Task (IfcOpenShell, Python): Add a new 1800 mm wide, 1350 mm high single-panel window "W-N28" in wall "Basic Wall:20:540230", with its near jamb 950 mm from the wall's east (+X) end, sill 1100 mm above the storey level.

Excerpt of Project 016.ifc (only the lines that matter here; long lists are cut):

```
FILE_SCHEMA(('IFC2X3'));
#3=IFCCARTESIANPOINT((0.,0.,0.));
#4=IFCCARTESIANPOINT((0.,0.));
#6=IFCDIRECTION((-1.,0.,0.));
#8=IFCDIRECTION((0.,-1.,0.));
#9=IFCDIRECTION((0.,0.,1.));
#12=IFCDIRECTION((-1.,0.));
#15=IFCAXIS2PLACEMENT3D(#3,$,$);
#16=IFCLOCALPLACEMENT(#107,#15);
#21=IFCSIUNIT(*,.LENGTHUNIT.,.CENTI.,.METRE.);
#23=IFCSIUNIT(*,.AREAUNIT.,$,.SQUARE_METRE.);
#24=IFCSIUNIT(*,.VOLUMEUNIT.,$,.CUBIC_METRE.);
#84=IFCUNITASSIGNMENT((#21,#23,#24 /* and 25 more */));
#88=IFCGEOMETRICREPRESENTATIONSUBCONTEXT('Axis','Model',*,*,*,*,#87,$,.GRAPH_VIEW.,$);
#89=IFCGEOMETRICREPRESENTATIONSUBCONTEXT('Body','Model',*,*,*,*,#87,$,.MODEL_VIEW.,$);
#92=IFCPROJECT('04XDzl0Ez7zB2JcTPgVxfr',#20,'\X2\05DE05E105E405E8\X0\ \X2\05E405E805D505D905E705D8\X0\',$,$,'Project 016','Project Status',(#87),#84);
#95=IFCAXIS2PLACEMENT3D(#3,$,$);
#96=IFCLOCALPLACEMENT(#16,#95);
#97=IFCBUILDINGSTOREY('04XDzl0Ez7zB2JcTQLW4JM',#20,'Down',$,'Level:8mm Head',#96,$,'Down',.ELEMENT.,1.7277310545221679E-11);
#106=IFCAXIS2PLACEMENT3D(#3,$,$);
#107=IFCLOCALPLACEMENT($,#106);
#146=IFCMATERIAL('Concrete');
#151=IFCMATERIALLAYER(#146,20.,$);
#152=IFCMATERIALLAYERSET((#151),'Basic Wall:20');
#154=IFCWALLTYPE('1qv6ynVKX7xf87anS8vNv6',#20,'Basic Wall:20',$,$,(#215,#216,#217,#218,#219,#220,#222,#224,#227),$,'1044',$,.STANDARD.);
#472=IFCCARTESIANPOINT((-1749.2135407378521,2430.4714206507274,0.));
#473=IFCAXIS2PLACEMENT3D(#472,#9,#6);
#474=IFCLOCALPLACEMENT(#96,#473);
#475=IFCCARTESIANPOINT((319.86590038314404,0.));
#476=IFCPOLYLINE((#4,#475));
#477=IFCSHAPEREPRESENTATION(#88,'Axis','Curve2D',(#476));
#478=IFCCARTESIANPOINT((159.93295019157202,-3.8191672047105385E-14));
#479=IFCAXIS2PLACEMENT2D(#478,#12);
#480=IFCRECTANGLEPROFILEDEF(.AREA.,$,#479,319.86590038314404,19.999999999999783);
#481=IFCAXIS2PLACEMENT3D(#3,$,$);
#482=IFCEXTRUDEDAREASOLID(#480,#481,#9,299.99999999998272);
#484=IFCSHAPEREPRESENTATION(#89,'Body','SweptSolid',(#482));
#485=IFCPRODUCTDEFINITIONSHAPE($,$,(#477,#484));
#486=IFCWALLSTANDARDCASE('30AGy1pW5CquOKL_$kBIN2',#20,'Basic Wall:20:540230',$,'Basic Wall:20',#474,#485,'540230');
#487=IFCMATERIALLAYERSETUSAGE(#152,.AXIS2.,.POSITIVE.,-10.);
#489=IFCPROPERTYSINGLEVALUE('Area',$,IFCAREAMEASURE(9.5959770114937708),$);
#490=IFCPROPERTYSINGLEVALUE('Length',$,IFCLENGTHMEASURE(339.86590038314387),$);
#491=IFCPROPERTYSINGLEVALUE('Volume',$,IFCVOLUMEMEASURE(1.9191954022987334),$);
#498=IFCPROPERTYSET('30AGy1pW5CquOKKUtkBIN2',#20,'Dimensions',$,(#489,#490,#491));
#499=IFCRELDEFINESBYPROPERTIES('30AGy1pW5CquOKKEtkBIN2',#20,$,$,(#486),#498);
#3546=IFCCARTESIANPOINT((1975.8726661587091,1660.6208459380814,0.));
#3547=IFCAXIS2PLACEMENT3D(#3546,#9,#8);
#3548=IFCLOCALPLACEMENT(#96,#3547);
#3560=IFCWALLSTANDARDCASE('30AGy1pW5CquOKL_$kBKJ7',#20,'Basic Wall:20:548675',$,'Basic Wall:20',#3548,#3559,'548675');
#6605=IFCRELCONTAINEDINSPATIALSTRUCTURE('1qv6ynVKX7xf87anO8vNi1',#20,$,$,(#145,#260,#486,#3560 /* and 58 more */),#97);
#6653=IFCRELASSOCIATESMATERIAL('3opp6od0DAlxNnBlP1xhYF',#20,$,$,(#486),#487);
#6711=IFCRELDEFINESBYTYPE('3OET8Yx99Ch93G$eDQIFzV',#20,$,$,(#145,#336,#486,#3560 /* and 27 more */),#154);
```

```python
import numpy as np
import ifcopenshell
import ifcopenshell.api.feature
import ifcopenshell.api.geometry
import ifcopenshell.api.pset
import ifcopenshell.api.root
import ifcopenshell.api.spatial
import ifcopenshell.api.type
import ifcopenshell.geom
import ifcopenshell.util.element
import ifcopenshell.util.placement
import ifcopenshell.util.representation
import ifcopenshell.util.shape
import ifcopenshell.util.unit

model = ifcopenshell.open("Project 016.ifc")
unit_scale = ifcopenshell.util.unit.calculate_unit_scale(model)
area_scale = ifcopenshell.util.unit.calculate_unit_scale(model, "AREAUNIT")
volume_scale = ifcopenshell.util.unit.calculate_unit_scale(model, "VOLUMEUNIT")
settings = ifcopenshell.geom.settings()


def volume(element):
    """Net volume in cubic metres, openings subtracted."""
    shape = ifcopenshell.geom.create_shape(settings, element)
    return ifcopenshell.util.shape.get_volume(shape.geometry)


wall = model.by_id(486)
storey = ifcopenshell.util.element.get_container(wall, ifc_class="IfcBuildingStorey")
context = ifcopenshell.util.representation.get_context(model, "Model", "Body", "MODEL_VIEW")
before = volume(wall)

width, height, from_end, sill = 1.8, 1.35, 0.95, 1.1  # metres

# The wall runs along its own X axis, and the end named is its -X end.
wall_shape = ifcopenshell.geom.create_shape(settings, wall)
x, y, z = ifcopenshell.util.shape.get_vertices(wall_shape.geometry).T
start = x.min() + from_end
face, thickness = float(y.min()), float(y.max() - y.min())
wall_matrix = ifcopenshell.util.placement.get_local_placement(wall.ObjectPlacement)
level = ifcopenshell.util.placement.get_local_placement(storey.ObjectPlacement)[2, 3]


def in_wall(x, y):
    """Placement at x, y metres in the wall's axes, at sill height."""
    matrix = wall_matrix.copy()
    matrix[:, 3] = wall_matrix @ np.array([x / unit_scale, y / unit_scale, 0.0, 1.0])
    matrix[2, 3] = level + sill / unit_scale
    return matrix


# Opening: a box that overshoots both wall faces by 50 mm.
opening = ifcopenshell.api.root.create_entity(model, ifc_class="IfcOpeningElement")
box = ifcopenshell.api.geometry.add_wall_representation(
    model, context=context, length=width, height=height, thickness=thickness + 0.1
)
ifcopenshell.api.geometry.assign_representation(model, product=opening, representation=box)
ifcopenshell.api.geometry.edit_object_placement(model, product=opening, matrix=in_wall(start, face - 0.05), is_si=False)
ifcopenshell.api.feature.add_feature(model, feature=opening, element=wall)

window = ifcopenshell.api.root.create_entity(model, ifc_class="IfcWindow", name="W-N28")
window.OverallWidth, window.OverallHeight = width / unit_scale, height / unit_scale
body = ifcopenshell.api.geometry.add_window_representation(
    model,
    context=context,
    overall_width=window.OverallWidth,
    overall_height=window.OverallHeight,
    partition_type="SINGLE_PANEL",
)
ifcopenshell.api.geometry.assign_representation(model, product=window, representation=body)
ifcopenshell.api.spatial.assign_container(model, products=[window], relating_structure=storey)
fills = ifcopenshell.api.feature.add_filling(model, opening=opening, element=window)
fills.OwnerHistory = window.OwnerHistory  # required in IFC2X3

# IFC2X3 keeps the operation on the window style.
style = ifcopenshell.api.root.create_entity(model, ifc_class="IfcWindowStyle", name="W-N28")
style.OperationType, style.ConstructionType = "SINGLE_PANEL", "NOTDEFINED"
style.ParameterTakesPrecedence = style.Sizeable = False
ifcopenshell.api.type.assign_type(model, related_objects=[window], relating_type=style)

# Centre the window in the wall's thickness.
ifcopenshell.api.geometry.edit_object_placement(model, product=window, matrix=in_wall(start, face), is_si=False)
window_shape = ifcopenshell.geom.create_shape(settings, window)
depth = ifcopenshell.util.shape.get_vertices(window_shape.geometry)[:, 1]
offset = face + thickness / 2 - (depth.min() + depth.max()) / 2
ifcopenshell.api.geometry.edit_object_placement(model, product=window, matrix=in_wall(start, offset), is_si=False)

after = volume(wall)

# Update the wall's stored quantities.
pset = model.by_id(ifcopenshell.util.element.get_pset(wall, "Dimensions", should_inherit=False)["id"])
ifcopenshell.api.pset.edit_pset(model, pset=pset, properties={
    "Area": model.create_entity("IfcAreaMeasure", after / thickness / area_scale),
    "Volume": model.create_entity("IfcVolumeMeasure", after / volume_scale),
})

print(f"wall volume {before:.3f} -> {after:.3f} m3")

model.write("Project 016_v2.ifc")
```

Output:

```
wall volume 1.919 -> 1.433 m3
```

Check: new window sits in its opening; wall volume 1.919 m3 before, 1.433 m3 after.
